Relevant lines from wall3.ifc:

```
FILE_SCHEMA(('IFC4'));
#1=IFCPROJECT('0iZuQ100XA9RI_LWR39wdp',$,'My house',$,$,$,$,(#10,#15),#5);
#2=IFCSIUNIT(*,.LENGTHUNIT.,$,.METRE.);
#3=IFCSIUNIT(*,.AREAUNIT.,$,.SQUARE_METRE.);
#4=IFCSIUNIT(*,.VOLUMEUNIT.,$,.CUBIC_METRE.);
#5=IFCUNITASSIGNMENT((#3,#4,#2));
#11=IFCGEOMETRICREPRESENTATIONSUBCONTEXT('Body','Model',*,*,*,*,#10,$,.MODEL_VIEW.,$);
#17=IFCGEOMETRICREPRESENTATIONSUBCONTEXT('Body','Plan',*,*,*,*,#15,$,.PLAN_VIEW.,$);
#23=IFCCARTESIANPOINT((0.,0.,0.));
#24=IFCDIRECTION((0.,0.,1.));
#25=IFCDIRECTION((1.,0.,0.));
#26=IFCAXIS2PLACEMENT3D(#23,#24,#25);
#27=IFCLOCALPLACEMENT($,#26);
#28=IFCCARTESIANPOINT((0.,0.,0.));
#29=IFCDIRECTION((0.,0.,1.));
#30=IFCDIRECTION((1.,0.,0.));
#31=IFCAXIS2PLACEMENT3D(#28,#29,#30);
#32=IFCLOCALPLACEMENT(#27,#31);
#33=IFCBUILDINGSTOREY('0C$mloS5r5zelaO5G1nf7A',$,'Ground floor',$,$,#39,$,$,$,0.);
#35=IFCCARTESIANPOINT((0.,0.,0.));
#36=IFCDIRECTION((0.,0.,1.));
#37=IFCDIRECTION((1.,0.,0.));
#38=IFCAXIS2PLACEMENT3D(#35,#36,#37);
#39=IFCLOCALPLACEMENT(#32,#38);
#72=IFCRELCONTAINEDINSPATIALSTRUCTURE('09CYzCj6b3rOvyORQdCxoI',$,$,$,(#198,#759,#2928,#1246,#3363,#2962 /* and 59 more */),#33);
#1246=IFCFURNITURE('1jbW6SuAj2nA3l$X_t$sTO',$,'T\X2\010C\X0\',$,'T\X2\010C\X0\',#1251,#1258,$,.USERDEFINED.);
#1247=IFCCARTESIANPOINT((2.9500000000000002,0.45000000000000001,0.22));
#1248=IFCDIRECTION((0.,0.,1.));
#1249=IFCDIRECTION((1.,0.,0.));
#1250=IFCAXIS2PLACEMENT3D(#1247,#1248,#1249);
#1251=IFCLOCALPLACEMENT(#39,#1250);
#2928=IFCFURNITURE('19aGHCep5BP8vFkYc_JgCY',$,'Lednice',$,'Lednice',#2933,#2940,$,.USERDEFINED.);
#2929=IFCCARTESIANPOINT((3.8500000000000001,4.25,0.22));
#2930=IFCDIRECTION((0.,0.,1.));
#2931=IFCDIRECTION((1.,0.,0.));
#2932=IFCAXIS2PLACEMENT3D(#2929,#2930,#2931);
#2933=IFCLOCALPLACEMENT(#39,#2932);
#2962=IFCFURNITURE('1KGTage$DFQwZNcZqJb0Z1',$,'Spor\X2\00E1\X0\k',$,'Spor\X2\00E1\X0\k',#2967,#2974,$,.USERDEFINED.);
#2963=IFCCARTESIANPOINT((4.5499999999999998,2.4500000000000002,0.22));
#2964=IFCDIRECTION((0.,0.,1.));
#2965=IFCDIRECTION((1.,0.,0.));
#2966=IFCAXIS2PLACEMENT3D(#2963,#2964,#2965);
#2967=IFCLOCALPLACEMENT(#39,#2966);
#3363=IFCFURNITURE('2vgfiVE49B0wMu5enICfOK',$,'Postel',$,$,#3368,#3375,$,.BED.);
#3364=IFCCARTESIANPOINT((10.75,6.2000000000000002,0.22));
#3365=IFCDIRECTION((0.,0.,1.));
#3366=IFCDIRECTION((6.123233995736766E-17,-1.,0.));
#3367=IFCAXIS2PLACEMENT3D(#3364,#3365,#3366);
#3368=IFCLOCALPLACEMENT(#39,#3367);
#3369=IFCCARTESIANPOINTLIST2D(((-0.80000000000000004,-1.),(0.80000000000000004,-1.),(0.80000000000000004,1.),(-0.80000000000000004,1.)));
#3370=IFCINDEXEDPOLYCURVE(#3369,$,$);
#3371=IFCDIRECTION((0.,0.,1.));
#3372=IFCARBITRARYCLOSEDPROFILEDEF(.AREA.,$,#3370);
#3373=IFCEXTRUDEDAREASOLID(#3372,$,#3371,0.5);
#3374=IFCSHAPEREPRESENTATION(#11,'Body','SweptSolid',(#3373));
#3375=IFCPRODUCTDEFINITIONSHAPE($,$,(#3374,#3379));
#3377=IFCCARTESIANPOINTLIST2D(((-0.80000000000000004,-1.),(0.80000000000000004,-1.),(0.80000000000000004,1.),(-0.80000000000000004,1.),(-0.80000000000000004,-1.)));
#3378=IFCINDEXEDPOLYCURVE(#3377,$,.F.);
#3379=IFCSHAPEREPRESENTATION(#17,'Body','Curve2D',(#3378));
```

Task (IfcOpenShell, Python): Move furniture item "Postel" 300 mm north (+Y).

```python
import ifcopenshell
import ifcopenshell.api.geometry
import ifcopenshell.util.placement
import ifcopenshell.util.unit

model = ifcopenshell.open("wall3.ifc")
unit_scale = ifcopenshell.util.unit.calculate_unit_scale(model)

item = model.by_guid("2vgfiVE49B0wMu5enICfOK")
matrix = ifcopenshell.util.placement.get_local_placement(item.ObjectPlacement)
matrix[1, 3] += 0.3 / unit_scale
ifcopenshell.api.geometry.edit_object_placement(model, product=item, matrix=matrix, is_si=False)

print(ifcopenshell.util.placement.get_local_placement(item.ObjectPlacement).round(3) + 0.0)

model.write("wall3_rev.ifc")
```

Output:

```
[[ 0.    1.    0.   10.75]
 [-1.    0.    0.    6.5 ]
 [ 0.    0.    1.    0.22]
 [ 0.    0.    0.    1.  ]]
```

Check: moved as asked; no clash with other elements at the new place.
